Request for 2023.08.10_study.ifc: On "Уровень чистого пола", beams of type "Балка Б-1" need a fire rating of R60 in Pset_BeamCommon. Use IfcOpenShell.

First a look at what the model holds.

```python
import ifcopenshell
import ifcopenshell.util.element

model = ifcopenshell.open("2023.08.10_study.ifc")
print(model.schema)
storey = next(s for s in model.by_type("IfcBuildingStorey") if s.Name == "Уровень чистого пола")
beams = [e for e in ifcopenshell.util.element.get_decomposition(storey) if e.is_a("IfcBeam")]
seen = {}
for e in beams:
    element_type = ifcopenshell.util.element.get_type(e)
    key = (element_type.Name if element_type != e and element_type else None, ifcopenshell.util.element.get_pset(e, "Pset_BeamCommon", "FireRating"))
    seen[key] = seen.get(key, 0) + 1
for (name, value), count in sorted(seen.items(), key=str):
    print(count, "x", name, "|", value)
```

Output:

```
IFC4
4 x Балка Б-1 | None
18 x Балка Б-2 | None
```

```python
import ifcopenshell
import ifcopenshell.api.pset
import ifcopenshell.util.element

model = ifcopenshell.open("2023.08.10_study.ifc")

storey = next(s for s in model.by_type("IfcBuildingStorey") if s.Name == "Уровень чистого пола")
beams = [e for e in ifcopenshell.util.element.get_decomposition(storey) if e.is_a("IfcBeam")]

count = 0
for e in beams:
    element_type = ifcopenshell.util.element.get_type(e)
    if element_type in (None, e) or element_type.Name != "Балка Б-1":
        continue
    # add_pset returns the element's existing set when there is one.
    pset = ifcopenshell.api.pset.add_pset(model, product=e, name="Pset_BeamCommon")
    ifcopenshell.api.pset.edit_pset(model, pset=pset, properties={"FireRating": "R60"})
    count += 1

print(count, "beams updated")

model.write("2023.08.10_study-out.ifc")
```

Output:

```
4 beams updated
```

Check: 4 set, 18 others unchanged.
